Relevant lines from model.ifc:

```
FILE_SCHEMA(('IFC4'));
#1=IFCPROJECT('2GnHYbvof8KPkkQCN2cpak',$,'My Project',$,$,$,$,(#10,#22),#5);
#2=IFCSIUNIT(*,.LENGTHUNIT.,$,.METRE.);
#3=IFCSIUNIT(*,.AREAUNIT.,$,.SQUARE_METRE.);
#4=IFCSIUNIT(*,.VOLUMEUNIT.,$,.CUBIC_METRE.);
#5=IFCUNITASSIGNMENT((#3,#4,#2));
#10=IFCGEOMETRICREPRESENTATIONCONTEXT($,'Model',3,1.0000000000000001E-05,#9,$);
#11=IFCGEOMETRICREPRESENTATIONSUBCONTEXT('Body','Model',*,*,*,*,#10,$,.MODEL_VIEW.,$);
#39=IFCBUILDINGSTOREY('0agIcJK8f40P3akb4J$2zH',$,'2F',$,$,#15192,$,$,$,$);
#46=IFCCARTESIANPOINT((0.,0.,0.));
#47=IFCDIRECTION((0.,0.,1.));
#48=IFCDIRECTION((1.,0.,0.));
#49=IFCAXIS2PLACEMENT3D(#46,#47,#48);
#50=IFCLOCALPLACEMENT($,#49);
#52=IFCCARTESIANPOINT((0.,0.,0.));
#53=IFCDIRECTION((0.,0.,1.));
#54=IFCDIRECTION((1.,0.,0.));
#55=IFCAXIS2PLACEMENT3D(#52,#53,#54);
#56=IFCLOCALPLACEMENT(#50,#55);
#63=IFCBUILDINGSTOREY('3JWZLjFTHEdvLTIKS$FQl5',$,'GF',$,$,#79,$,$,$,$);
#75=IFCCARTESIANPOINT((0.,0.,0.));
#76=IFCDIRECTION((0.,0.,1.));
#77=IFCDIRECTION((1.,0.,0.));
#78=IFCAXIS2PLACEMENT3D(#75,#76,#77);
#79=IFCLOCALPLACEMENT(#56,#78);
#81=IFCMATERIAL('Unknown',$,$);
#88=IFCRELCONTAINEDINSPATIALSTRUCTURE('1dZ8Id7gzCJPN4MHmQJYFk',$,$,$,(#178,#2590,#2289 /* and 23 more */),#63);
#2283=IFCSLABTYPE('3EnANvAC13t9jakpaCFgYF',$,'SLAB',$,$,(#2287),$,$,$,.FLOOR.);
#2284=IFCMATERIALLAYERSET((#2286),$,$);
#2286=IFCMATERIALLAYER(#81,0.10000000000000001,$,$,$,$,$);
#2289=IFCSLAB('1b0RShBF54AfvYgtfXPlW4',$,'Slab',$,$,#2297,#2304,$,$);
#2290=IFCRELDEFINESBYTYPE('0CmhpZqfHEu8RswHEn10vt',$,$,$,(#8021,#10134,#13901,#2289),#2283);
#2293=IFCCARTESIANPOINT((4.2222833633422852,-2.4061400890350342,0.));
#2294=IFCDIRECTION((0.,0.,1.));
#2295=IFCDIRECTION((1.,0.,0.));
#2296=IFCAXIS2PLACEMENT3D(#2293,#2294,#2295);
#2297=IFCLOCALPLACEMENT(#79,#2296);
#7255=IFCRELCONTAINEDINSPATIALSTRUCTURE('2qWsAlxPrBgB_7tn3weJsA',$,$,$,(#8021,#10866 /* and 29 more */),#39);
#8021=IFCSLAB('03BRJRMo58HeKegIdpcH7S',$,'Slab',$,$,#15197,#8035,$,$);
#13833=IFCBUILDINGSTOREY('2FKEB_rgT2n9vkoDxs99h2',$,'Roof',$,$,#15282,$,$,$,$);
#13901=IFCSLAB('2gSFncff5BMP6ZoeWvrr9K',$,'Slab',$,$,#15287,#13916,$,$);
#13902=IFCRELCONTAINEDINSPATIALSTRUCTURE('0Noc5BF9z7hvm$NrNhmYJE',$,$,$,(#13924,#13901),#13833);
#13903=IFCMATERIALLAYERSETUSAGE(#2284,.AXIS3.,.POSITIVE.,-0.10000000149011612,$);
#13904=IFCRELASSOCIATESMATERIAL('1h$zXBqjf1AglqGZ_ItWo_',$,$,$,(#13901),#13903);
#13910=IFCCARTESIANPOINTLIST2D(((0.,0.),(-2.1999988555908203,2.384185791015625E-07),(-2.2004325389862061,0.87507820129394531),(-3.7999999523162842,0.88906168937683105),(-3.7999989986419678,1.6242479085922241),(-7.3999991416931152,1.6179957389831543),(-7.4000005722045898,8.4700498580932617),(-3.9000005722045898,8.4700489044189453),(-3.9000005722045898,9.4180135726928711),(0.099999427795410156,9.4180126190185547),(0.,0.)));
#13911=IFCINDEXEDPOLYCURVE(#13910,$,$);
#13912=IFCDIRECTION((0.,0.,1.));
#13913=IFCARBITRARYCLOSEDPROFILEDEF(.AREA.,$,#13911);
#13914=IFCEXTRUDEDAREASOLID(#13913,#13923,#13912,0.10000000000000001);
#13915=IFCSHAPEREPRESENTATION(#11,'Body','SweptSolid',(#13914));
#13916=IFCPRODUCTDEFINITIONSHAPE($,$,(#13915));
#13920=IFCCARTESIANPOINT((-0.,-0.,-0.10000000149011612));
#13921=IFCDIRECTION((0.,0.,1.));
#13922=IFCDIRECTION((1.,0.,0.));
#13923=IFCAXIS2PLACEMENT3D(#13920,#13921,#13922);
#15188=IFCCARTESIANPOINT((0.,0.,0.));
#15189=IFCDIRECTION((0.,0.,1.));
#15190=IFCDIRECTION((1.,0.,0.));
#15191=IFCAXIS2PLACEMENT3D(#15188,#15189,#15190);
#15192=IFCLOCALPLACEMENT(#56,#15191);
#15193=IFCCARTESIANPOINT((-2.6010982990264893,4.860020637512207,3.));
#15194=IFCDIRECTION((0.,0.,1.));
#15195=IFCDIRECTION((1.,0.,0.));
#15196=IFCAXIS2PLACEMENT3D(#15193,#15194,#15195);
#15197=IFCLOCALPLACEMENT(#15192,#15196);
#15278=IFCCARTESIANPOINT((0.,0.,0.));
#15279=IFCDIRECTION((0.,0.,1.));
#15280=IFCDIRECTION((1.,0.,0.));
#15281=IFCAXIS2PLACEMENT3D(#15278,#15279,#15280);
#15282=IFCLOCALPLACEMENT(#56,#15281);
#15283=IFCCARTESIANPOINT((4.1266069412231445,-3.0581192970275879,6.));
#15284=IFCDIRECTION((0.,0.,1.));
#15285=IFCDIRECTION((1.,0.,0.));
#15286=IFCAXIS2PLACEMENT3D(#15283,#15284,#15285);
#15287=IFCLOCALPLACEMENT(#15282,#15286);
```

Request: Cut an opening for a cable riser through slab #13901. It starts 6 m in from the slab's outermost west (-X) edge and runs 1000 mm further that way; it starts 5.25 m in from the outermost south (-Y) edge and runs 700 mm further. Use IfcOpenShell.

```python
import numpy as np
import ifcopenshell
import ifcopenshell.api.feature
import ifcopenshell.api.geometry
import ifcopenshell.api.root
import ifcopenshell.geom
import ifcopenshell.util.placement
import ifcopenshell.util.representation
import ifcopenshell.util.shape
import ifcopenshell.util.unit

model = ifcopenshell.open("model.ifc")
unit_scale = ifcopenshell.util.unit.calculate_unit_scale(model)
settings = ifcopenshell.geom.settings()


def volume(element):
    """Net volume in cubic metres, openings subtracted."""
    shape = ifcopenshell.geom.create_shape(settings, element)
    return ifcopenshell.util.shape.get_volume(shape.geometry)


slab = model.by_id(13901)
before = volume(slab)

# Extent in the slab's own axes, in metres. The edges named are its -X and -Y sides.
slab_shape = ifcopenshell.geom.create_shape(settings, slab)
vertices = ifcopenshell.util.shape.get_vertices(slab_shape.geometry)
x_min, y_min, bottom = vertices.min(axis=0)
top = vertices[:, 2].max()

opening = ifcopenshell.api.root.create_entity(model, ifc_class="IfcOpeningElement", name="Cable riser opening", predefined_type="OPENING")
context = ifcopenshell.util.representation.get_context(model, "Model", "Body", "MODEL_VIEW")
width, depth = 1, 0.7
outline = [(0.0, 0.0), (width, 0.0), (width, depth), (0.0, depth), (0.0, 0.0)]
# Overshoot both faces by 50 mm so the cut is clean.
shape = ifcopenshell.api.geometry.add_slab_representation(
    model, context=context, depth=top - bottom + 0.1, polyline=outline
)
ifcopenshell.api.geometry.assign_representation(model, product=opening, representation=shape)

matrix = ifcopenshell.util.placement.get_local_placement(slab.ObjectPlacement)
matrix[:, 3] = matrix @ np.append(np.array([x_min + 6, y_min + 5.25, bottom - 0.05]) / unit_scale, 1.0)
ifcopenshell.api.geometry.edit_object_placement(model, product=opening, matrix=matrix, is_si=False)
ifcopenshell.api.feature.add_feature(model, feature=opening, element=slab)

after = volume(slab)

print(f"slab volume {before:.3f} -> {after:.3f} m3")

model.write("model-out.ifc")
```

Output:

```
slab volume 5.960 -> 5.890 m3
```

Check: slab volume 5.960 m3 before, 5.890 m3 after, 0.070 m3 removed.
